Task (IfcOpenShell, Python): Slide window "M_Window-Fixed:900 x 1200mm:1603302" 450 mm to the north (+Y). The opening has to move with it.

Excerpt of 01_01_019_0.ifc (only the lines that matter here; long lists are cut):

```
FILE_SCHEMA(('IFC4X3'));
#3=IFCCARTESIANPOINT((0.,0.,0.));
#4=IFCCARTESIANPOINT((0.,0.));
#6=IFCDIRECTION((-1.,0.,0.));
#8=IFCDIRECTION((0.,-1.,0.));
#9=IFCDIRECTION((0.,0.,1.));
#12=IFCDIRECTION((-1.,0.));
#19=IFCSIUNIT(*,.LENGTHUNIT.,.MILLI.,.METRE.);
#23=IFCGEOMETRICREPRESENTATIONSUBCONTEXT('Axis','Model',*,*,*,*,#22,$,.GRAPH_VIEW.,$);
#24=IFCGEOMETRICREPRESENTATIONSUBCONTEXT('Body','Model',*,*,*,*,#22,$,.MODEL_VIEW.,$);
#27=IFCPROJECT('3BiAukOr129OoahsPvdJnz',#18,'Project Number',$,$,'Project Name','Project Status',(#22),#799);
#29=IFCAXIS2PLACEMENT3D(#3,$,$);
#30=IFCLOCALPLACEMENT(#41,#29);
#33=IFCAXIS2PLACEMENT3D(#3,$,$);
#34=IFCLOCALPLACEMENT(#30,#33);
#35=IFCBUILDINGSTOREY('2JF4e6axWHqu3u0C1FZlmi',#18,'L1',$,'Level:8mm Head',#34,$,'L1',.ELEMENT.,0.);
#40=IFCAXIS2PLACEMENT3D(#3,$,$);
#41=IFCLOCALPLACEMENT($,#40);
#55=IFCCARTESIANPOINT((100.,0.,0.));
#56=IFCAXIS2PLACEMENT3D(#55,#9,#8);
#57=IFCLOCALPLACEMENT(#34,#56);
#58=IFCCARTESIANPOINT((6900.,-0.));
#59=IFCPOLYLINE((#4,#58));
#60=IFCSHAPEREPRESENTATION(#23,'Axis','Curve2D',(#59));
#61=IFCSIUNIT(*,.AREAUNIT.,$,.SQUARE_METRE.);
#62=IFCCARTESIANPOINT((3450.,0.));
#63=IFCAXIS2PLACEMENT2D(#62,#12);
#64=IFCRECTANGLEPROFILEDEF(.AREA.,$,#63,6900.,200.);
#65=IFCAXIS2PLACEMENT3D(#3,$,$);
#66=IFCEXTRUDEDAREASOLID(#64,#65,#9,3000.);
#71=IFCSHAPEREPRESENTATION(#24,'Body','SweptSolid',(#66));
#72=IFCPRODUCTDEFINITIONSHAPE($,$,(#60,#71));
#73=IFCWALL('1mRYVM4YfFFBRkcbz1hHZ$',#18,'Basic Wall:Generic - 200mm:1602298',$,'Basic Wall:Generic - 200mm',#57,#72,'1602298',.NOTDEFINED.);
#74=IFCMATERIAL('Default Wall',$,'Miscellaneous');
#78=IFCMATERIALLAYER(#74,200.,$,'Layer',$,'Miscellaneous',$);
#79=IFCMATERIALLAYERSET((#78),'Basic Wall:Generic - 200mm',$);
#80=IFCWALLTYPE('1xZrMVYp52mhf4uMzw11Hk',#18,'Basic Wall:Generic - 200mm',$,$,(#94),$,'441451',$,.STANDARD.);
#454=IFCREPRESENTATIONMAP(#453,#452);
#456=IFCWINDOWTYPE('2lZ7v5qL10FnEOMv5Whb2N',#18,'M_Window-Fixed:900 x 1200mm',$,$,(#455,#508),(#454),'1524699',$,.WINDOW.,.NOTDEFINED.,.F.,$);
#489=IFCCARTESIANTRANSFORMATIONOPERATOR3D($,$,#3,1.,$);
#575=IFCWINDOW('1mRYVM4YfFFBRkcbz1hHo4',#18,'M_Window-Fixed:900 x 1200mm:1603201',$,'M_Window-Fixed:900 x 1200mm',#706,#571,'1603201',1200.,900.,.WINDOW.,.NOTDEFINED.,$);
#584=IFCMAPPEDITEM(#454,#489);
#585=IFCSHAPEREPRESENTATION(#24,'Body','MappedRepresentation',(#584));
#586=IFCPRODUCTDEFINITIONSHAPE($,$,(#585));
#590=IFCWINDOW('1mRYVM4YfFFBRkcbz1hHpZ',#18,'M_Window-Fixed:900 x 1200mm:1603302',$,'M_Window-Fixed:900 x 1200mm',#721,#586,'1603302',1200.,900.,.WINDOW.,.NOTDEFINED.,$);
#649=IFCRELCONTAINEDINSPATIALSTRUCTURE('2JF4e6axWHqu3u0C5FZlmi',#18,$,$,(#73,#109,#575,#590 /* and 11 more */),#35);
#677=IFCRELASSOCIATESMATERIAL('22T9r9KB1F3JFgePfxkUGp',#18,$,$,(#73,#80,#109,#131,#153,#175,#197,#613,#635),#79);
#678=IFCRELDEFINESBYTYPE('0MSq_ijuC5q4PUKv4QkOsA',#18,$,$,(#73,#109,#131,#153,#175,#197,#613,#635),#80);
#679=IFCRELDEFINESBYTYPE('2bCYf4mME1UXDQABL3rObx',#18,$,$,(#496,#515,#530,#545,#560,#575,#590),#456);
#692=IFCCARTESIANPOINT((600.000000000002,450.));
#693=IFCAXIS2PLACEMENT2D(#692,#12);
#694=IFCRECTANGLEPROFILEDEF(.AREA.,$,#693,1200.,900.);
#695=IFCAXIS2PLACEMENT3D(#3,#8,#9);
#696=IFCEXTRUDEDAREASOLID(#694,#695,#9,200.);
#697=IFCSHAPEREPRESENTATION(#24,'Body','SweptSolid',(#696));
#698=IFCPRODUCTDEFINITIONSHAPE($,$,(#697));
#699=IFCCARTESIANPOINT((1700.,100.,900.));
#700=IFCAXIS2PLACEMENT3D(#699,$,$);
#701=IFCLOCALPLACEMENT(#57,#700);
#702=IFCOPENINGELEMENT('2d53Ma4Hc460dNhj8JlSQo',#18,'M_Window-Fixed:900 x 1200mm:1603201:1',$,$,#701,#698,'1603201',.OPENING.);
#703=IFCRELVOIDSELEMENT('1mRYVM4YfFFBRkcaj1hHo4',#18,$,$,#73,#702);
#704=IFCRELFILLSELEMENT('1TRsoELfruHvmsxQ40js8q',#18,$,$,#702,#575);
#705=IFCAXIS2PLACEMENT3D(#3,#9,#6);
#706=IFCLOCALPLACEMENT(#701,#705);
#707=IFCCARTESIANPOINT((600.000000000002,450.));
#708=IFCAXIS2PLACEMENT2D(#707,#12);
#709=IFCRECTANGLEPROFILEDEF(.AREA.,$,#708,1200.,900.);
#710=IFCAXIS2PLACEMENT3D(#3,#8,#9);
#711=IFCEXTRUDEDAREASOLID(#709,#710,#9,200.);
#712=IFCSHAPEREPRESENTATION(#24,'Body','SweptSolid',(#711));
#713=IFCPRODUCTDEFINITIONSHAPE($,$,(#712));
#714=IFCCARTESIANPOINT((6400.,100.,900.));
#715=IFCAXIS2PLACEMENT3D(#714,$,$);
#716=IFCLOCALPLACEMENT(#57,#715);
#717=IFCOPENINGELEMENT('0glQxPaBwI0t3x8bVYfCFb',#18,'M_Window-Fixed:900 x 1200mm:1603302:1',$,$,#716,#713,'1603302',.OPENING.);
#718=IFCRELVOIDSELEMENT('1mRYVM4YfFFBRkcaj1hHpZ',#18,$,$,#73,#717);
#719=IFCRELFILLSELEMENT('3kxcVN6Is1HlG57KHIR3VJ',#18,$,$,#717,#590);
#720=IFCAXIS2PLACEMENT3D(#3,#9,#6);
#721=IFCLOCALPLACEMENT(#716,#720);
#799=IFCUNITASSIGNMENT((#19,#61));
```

```python
import ifcopenshell
import ifcopenshell.api.geometry
import ifcopenshell.util.placement
import ifcopenshell.util.unit

model = ifcopenshell.open("01_01_019_0.ifc")
unit_scale = ifcopenshell.util.unit.calculate_unit_scale(model)

window = model.by_guid("1mRYVM4YfFFBRkcbz1hHpZ")
opening = window.FillsVoids[0].RelatingOpeningElement
wall = opening.VoidsElements[0].RelatingBuildingElement

wall_matrix = ifcopenshell.util.placement.get_local_placement(wall.ObjectPlacement)
shift = wall_matrix[:3, 0] * -0.45 / unit_scale
before = ifcopenshell.util.placement.get_local_placement(window.ObjectPlacement)[:3, 3].copy()

# The window is placed relative to its opening, so it follows when the opening moves.
matrix = ifcopenshell.util.placement.get_local_placement(opening.ObjectPlacement)
matrix[:3, 3] += shift
ifcopenshell.api.geometry.edit_object_placement(
    model, product=opening, matrix=matrix, is_si=False, should_transform_children=True
)

after = ifcopenshell.util.placement.get_local_placement(window.ObjectPlacement)[:3, 3]
print("window moved by", (after - before).round(3) + 0.0)

model.write("01_01_019_0_v2.ifc")
```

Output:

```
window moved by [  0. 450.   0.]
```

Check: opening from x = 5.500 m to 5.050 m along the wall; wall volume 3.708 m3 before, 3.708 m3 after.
